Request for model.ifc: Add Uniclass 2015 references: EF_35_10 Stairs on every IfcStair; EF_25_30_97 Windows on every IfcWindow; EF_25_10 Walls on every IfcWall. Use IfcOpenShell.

First a look at what the model holds.

```python
import ifcopenshell

model = ifcopenshell.open("model.ifc")
print(model.schema)
print("classifications:", [c.Name for c in model.by_type("IfcClassification")])
for ifc_class in ("IfcDoor", "IfcRoof", "IfcStair", "IfcWall", "IfcWindow"):
    print(ifc_class, len(model.by_type(ifc_class)))
```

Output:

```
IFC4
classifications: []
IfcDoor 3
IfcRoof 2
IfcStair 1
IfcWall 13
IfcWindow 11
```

```python
import ifcopenshell
import ifcopenshell.api.classification

model = ifcopenshell.open("model.ifc")

system = ifcopenshell.api.classification.add_classification(model, classification="Uniclass 2015")

codes = {
    "IfcStair": ("EF_35_10", "Stairs"),
    "IfcWindow": ("EF_25_30_97", "Windows"),
    "IfcWall": ("EF_25_10", "Walls"),
}
for ifc_class, (code, name) in codes.items():
    products = model.by_type(ifc_class)
    ifcopenshell.api.classification.add_reference(
        model, products=products, classification=system, identification=code, name=name
    )
    print(code, len(products))

model.write("model_updated.ifc")
```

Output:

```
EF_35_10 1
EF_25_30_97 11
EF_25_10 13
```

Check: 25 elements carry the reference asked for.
